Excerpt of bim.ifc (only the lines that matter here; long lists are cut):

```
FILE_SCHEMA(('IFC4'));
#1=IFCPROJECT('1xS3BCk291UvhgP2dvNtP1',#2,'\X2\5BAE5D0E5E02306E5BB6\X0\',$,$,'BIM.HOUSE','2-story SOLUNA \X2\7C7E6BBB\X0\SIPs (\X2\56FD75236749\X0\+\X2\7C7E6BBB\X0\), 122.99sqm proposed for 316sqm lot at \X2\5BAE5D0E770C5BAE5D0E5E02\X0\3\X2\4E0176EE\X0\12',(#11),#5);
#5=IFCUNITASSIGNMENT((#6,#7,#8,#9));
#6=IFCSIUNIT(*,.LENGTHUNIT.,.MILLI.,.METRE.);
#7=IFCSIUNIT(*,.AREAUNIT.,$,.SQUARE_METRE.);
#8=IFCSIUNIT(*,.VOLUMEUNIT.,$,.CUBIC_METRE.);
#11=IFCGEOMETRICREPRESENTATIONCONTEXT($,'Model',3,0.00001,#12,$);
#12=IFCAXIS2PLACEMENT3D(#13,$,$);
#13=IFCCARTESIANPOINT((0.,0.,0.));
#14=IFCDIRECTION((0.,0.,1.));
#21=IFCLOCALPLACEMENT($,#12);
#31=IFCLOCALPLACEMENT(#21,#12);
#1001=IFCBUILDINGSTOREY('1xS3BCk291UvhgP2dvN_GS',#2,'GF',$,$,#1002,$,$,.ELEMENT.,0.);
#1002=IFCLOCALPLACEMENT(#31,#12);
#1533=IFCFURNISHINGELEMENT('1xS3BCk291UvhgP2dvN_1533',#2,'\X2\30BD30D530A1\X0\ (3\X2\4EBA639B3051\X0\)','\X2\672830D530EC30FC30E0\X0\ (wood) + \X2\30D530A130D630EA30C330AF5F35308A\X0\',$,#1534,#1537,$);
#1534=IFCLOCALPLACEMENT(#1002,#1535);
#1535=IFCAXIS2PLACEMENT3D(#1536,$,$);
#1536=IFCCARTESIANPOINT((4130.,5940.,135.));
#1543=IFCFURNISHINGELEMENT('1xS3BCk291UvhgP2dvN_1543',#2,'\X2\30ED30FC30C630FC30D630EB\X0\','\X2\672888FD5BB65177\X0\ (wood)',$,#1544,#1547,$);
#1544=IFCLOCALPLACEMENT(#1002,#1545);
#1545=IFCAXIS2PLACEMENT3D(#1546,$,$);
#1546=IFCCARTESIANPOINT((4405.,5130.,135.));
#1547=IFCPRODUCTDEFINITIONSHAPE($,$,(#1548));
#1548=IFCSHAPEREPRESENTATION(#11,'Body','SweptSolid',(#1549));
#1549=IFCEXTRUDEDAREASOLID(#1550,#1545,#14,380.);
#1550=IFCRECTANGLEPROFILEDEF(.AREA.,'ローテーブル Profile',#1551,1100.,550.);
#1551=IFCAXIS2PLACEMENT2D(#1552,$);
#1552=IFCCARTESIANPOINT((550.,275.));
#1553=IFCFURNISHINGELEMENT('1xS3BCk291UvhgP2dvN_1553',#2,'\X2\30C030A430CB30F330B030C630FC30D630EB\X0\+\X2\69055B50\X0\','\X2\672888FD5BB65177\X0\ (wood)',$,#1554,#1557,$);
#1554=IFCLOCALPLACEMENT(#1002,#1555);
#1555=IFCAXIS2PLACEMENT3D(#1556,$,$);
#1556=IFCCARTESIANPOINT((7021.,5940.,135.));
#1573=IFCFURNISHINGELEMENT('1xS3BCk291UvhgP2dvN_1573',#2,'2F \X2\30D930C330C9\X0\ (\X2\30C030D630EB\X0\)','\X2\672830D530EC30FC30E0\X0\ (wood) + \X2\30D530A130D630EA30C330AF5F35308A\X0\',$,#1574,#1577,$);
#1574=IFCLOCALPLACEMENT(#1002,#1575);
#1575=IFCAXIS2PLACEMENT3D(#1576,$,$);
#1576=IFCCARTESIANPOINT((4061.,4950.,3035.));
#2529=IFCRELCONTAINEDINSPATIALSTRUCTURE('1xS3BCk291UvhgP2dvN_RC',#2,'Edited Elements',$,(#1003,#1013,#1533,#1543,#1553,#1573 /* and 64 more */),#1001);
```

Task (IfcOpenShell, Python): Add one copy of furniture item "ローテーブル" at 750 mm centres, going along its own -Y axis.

```python
import ifcopenshell
import ifcopenshell.api.geometry
import ifcopenshell.api.root
import ifcopenshell.util.element
import ifcopenshell.util.placement
import ifcopenshell.util.unit

model = ifcopenshell.open("bim.ifc")
unit_scale = ifcopenshell.util.unit.calculate_unit_scale(model)


def reuse_history(source, copy):
    """copy_class also copies each property set's owner history, people and application; keep the originals."""
    for rel in copy.IsDefinedBy:
        if rel.is_a("IfcRelDefinesByProperties") and (history := rel.RelatingPropertyDefinition.OwnerHistory):
            rel.RelatingPropertyDefinition.OwnerHistory = source.OwnerHistory
            ifcopenshell.util.element.remove_deep2(model, history)


source = model.by_guid("1xS3BCk291UvhgP2dvN_1543")
base = ifcopenshell.util.placement.get_local_placement(source.ObjectPlacement)
step = -base[:3, 1] * 0.75 / unit_scale

for i in range(1, 2):
    copy = ifcopenshell.api.root.copy_class(model, product=source)
    copy.Representation = ifcopenshell.util.element.copy_deep(
        model, source.Representation, exclude=["IfcGeometricRepresentationContext", "IfcRepresentationMap"]
    )
    reuse_history(source, copy)
    matrix = base.copy()
    matrix[:3, 3] += i * step
    print("added at", matrix[:3, 3].round(3) + 0.0)
    ifcopenshell.api.geometry.edit_object_placement(model, product=copy, matrix=matrix, is_si=False)

model.write("bim_v2.ifc")
```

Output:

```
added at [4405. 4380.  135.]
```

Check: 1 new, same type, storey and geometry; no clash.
